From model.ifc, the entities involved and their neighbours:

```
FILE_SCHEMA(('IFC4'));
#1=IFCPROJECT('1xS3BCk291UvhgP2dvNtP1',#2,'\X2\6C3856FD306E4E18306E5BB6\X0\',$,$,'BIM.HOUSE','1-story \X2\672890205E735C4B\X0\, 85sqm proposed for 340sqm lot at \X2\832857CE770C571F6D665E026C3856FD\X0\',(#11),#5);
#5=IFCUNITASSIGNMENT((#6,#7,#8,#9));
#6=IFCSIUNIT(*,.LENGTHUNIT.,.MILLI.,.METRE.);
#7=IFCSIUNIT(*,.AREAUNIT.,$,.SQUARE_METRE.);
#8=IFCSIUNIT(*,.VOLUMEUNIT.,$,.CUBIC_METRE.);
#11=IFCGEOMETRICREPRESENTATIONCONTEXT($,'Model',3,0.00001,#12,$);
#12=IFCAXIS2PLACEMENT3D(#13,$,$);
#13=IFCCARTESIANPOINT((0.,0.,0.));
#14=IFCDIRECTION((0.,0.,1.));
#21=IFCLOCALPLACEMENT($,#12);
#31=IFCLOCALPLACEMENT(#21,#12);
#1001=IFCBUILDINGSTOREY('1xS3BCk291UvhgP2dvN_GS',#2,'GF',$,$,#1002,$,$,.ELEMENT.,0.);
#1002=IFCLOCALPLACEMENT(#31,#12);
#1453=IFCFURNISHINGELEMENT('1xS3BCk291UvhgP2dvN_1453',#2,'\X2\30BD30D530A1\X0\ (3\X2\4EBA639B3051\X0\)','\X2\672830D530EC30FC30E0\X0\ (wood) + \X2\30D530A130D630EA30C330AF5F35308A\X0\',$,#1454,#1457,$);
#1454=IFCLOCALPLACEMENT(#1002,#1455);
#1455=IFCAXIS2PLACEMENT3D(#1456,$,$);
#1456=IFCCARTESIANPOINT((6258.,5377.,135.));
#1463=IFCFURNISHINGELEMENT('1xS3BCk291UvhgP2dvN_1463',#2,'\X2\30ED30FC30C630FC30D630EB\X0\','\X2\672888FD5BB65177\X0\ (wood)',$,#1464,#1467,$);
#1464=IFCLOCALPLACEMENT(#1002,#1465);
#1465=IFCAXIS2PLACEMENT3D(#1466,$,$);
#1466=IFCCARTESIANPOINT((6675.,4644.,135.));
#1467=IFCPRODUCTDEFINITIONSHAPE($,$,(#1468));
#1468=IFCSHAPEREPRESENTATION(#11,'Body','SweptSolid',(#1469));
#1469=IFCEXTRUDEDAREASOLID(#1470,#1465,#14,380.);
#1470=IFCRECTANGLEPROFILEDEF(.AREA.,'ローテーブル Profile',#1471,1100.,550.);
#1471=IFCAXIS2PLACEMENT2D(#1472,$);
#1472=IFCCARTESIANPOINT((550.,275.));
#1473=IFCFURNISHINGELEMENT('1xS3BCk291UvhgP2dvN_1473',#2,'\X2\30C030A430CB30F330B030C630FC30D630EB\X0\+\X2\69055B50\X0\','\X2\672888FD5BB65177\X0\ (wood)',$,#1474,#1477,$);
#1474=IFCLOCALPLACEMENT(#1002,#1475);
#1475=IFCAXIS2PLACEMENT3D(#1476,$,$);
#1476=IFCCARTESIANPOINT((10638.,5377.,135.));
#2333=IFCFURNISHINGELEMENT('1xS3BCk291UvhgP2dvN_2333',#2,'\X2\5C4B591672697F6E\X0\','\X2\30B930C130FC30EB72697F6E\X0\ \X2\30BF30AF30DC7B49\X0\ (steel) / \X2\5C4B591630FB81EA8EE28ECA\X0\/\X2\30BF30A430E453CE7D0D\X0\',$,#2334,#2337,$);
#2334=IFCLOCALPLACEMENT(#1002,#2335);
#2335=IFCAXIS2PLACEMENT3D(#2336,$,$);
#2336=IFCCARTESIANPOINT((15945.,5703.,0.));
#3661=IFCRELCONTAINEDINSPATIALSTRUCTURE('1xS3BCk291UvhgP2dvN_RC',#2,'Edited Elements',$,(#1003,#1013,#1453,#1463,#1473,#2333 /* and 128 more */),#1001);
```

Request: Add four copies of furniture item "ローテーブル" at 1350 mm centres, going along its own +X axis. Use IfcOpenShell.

```python
import ifcopenshell
import ifcopenshell.api.geometry
import ifcopenshell.api.root
import ifcopenshell.util.element
import ifcopenshell.util.placement
import ifcopenshell.util.unit

model = ifcopenshell.open("model.ifc")
unit_scale = ifcopenshell.util.unit.calculate_unit_scale(model)


def reuse_history(source, copy):
    """copy_class also copies each property set's owner history, people and application; keep the originals."""
    for rel in copy.IsDefinedBy:
        if rel.is_a("IfcRelDefinesByProperties") and (history := rel.RelatingPropertyDefinition.OwnerHistory):
            rel.RelatingPropertyDefinition.OwnerHistory = source.OwnerHistory
            ifcopenshell.util.element.remove_deep2(model, history)


source = model.by_id(1463)
base = ifcopenshell.util.placement.get_local_placement(source.ObjectPlacement)
step = base[:3, 0] * 1.35 / unit_scale

for i in range(1, 5):
    copy = ifcopenshell.api.root.copy_class(model, product=source)
    copy.Representation = ifcopenshell.util.element.copy_deep(
        model, source.Representation, exclude=["IfcGeometricRepresentationContext", "IfcRepresentationMap"]
    )
    reuse_history(source, copy)
    matrix = base.copy()
    matrix[:3, 3] += i * step
    print("added at", matrix[:3, 3].round(3) + 0.0)
    ifcopenshell.api.geometry.edit_object_placement(model, product=copy, matrix=matrix, is_si=False)

model.write("model_updated.ifc")
```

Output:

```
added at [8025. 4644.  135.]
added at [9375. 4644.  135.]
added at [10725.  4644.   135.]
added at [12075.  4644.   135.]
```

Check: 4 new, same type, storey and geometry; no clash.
